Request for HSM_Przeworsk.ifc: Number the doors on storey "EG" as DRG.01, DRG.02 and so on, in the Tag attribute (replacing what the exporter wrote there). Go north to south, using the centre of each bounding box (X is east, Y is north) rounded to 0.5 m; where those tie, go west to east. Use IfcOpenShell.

First a look at what the model holds.

```python
import ifcopenshell
import ifcopenshell.util.element
import ifcopenshell.util.placement

model = ifcopenshell.open("HSM_Przeworsk.ifc")
print(model.schema)
storey = next(s for s in model.by_type("IfcBuildingStorey") if s.Name == "EG")
doors = [e for e in ifcopenshell.util.element.get_decomposition(storey) if e.is_a("IfcDoor")]
for e in sorted(doors, key=lambda e: e.id()):
    origin = ifcopenshell.util.placement.get_local_placement(e.ObjectPlacement)[:3, 3]
    print(e.id(), e.Tag, e.Name, origin.round(2) + 0.0, sep=" | ")
```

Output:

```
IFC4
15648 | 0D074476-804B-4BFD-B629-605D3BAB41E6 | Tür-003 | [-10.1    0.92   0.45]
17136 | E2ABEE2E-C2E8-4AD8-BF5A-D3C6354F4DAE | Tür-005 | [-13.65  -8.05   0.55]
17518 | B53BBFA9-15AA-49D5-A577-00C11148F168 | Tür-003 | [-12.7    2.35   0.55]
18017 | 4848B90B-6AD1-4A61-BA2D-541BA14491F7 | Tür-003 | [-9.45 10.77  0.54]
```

```python
import ifcopenshell
import ifcopenshell.geom
import ifcopenshell.util.element
import ifcopenshell.util.shape

model = ifcopenshell.open("HSM_Przeworsk.ifc")
settings = ifcopenshell.geom.settings()
settings.set("use-world-coords", True)


def centre(element):
    shape = ifcopenshell.geom.create_shape(settings, element)
    return ifcopenshell.util.shape.get_bbox_centroid(shape.geometry)


storey = next(s for s in model.by_type("IfcBuildingStorey") if s.Name == "EG")
doors = [e for e in ifcopenshell.util.element.get_decomposition(storey) if e.is_a("IfcDoor")]

# Insertion points can sit at a corner or the storey origin, so sort by the geometry (in metres).
centres = {e: centre(e) for e in doors}
doors.sort(key=lambda e: (-round(centres[e][1] / 0.5), centres[e][0]))

for i, e in enumerate(doors, start=1):
    number = f"DRG.{i:02d}"
    e.Tag = number
    print(e.id(), number)

model.write("HSM_Przeworsk_updated.ifc")
```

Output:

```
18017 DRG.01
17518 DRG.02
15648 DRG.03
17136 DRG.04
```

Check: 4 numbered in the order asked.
